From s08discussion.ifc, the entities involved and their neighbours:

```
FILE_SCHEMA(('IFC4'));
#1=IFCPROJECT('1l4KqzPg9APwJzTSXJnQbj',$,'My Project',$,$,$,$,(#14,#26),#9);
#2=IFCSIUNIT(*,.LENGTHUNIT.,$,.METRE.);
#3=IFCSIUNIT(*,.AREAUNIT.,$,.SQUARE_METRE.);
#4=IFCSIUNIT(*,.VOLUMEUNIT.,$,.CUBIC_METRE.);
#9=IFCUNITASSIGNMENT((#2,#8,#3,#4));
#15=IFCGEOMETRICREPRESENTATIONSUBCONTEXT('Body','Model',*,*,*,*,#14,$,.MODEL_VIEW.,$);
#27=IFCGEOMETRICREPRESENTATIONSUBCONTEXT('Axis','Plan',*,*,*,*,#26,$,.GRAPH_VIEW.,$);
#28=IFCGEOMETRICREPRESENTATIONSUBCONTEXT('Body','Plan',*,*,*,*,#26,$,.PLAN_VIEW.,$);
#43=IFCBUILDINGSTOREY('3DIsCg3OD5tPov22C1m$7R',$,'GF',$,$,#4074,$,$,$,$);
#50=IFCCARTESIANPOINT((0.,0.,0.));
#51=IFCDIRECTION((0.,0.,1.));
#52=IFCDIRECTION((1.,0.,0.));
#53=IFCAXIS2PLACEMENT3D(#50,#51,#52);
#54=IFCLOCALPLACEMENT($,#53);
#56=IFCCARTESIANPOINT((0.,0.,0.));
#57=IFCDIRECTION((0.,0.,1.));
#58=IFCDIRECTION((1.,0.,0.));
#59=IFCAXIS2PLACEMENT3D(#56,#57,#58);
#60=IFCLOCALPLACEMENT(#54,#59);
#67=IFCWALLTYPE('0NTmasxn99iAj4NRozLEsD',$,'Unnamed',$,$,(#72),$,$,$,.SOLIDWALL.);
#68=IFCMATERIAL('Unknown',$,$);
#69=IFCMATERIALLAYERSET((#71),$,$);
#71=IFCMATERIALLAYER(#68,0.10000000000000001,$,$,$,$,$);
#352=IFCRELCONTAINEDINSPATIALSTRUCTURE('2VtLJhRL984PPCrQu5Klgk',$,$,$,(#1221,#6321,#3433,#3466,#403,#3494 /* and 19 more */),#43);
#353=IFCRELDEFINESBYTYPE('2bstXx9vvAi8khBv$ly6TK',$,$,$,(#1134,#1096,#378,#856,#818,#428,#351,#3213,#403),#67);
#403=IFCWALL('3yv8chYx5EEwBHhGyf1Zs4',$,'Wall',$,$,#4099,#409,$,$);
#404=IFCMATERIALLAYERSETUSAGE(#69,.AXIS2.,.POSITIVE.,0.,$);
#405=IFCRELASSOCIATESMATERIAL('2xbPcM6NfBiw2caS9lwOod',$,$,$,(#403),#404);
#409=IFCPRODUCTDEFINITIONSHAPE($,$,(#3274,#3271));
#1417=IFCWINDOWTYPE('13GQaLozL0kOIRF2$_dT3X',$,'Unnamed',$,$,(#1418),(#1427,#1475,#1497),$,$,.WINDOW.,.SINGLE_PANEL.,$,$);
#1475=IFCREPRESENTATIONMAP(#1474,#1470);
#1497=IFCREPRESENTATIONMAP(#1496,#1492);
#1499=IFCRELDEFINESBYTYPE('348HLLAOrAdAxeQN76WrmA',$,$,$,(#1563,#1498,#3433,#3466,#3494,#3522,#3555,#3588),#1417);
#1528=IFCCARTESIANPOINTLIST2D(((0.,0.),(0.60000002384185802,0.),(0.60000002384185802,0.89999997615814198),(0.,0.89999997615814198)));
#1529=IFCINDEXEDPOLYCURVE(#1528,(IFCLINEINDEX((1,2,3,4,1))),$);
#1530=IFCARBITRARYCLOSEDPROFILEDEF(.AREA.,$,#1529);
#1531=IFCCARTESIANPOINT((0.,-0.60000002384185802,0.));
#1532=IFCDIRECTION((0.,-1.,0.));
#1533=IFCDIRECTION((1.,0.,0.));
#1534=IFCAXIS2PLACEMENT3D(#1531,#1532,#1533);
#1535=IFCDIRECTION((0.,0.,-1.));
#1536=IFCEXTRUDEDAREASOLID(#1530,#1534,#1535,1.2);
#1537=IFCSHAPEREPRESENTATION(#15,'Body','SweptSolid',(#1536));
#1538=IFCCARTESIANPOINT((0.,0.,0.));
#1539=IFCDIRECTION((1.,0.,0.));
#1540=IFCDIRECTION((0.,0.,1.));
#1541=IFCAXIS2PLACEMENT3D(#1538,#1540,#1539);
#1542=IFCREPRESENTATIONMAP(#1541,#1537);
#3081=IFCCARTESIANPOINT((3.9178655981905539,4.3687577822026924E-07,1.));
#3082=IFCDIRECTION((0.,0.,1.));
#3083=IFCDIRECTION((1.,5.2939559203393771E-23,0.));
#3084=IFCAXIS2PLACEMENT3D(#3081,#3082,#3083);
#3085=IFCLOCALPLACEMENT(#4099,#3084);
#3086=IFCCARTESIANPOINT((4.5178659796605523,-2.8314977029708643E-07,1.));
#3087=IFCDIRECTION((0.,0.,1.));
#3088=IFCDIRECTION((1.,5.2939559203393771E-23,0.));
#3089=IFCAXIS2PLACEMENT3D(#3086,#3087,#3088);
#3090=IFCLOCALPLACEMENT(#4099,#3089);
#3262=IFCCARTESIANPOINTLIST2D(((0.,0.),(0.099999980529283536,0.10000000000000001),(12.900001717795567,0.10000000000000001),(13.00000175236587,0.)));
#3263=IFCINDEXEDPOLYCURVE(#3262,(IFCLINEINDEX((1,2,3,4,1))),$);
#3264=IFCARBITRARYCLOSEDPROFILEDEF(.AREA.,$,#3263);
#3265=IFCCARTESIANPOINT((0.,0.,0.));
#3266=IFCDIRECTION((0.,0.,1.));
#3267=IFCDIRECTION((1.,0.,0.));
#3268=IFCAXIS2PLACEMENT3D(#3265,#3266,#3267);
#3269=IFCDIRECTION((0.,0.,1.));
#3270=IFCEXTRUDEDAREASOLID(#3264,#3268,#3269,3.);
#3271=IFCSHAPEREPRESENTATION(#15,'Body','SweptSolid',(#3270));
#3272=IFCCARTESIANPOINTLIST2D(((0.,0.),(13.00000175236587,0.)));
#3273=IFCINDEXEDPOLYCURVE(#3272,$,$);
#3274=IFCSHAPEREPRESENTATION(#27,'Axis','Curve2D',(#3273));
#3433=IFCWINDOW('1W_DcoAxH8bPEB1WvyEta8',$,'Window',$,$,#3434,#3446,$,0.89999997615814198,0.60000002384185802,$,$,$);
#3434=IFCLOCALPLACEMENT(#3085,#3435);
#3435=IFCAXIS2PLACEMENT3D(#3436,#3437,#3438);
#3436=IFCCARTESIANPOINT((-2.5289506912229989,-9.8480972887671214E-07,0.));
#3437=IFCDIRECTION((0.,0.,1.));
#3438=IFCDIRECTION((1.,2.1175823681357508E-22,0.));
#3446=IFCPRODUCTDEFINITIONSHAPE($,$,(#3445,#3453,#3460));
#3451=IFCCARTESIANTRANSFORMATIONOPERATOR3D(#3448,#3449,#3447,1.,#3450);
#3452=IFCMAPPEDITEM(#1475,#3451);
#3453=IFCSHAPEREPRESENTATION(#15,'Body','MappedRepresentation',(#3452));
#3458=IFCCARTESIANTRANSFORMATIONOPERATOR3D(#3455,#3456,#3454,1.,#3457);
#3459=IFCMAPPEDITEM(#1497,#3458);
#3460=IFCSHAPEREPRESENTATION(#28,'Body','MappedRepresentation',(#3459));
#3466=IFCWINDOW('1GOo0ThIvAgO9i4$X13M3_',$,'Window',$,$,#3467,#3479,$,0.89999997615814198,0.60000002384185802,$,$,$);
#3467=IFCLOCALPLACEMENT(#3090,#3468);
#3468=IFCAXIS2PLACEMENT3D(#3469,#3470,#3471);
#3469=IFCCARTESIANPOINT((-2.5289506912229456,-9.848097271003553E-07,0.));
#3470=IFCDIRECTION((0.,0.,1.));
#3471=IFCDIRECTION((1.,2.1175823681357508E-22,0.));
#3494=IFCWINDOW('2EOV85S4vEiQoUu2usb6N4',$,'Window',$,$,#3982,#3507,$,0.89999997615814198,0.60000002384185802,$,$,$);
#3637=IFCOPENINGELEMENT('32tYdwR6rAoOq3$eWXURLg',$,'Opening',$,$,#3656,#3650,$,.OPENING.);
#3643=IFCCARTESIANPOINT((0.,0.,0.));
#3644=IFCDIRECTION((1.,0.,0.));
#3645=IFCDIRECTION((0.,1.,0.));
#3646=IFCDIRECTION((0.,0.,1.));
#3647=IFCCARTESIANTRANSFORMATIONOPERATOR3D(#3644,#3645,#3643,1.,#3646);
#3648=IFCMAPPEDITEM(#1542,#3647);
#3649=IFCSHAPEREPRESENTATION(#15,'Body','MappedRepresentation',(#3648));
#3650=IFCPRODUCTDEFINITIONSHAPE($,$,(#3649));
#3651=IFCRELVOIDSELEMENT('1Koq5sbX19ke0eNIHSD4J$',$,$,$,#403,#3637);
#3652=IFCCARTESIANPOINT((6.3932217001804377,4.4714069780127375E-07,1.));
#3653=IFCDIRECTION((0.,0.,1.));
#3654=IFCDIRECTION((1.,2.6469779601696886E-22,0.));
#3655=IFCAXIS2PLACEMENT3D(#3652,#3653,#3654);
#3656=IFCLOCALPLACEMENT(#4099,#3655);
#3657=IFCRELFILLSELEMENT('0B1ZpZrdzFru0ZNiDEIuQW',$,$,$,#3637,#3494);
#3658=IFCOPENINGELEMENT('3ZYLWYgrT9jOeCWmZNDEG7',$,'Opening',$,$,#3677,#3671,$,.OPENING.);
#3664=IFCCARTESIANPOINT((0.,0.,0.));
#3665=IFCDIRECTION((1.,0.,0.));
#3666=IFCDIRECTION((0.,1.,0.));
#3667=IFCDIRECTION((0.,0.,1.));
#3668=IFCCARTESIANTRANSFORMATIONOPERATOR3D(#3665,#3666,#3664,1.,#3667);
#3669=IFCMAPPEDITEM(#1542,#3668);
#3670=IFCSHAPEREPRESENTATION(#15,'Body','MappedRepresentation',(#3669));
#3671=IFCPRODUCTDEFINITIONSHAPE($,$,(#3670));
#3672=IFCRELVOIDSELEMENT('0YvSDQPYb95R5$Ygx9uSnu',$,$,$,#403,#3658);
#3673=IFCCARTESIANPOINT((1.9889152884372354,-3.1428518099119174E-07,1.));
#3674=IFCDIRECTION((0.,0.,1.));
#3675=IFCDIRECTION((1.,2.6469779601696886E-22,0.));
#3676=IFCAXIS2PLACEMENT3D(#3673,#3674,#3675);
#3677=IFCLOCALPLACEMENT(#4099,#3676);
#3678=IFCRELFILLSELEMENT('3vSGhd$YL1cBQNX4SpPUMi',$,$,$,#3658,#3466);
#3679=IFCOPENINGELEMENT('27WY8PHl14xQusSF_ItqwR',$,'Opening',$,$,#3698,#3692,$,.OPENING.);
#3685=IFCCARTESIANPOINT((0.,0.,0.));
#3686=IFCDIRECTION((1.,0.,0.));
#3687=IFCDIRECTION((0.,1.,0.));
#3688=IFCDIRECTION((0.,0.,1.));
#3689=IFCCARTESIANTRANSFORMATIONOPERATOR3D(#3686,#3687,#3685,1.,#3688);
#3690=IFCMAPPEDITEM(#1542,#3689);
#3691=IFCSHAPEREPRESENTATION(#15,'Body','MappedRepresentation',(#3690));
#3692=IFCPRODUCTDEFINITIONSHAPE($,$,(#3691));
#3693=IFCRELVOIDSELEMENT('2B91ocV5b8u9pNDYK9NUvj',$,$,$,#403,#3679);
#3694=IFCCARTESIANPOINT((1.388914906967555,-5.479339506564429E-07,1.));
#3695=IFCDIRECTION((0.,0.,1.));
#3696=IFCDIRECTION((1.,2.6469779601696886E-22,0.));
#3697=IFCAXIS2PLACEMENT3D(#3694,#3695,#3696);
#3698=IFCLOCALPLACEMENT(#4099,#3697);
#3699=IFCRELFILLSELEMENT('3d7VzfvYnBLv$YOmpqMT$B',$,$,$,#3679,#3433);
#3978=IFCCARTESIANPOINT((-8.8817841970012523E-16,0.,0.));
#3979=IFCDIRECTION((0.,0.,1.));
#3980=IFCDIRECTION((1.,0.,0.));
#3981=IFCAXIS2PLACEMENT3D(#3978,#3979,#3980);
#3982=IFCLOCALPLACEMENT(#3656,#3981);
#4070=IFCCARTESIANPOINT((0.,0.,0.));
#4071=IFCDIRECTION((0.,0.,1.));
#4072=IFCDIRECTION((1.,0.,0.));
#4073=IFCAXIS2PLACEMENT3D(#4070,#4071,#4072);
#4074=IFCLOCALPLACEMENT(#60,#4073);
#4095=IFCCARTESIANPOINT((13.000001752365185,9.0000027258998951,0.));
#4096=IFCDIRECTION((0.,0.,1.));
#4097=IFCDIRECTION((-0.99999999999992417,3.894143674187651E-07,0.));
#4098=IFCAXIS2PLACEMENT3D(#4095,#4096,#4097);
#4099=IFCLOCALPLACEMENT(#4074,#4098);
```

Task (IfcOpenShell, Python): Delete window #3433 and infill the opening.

```python
import ifcopenshell
import ifcopenshell.api.feature
import ifcopenshell.api.root
import ifcopenshell.geom
import ifcopenshell.util.shape

model = ifcopenshell.open("s08discussion.ifc")
settings = ifcopenshell.geom.settings()


def volume(element):
    """Net volume in cubic metres, openings subtracted."""
    shape = ifcopenshell.geom.create_shape(settings, element)
    return ifcopenshell.util.shape.get_volume(shape.geometry)


window = model.by_guid("1W_DcoAxH8bPEB1WvyEta8")
opening = window.FillsVoids[0].RelatingOpeningElement
wall = opening.VoidsElements[0].RelatingBuildingElement
before = volume(wall)

ifcopenshell.api.root.remove_product(model, product=window)
ifcopenshell.api.feature.remove_feature(model, feature=opening)

after = volume(wall)

print(f"wall volume {before:.3f} -> {after:.3f} m3")

model.write("s08discussion_updated.ifc")
```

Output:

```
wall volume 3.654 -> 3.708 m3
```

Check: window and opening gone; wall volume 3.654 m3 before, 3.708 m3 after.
